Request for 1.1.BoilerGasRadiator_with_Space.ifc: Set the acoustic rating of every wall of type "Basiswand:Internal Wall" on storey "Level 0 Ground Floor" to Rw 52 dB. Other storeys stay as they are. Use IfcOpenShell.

First a look at what the model holds.

```python
import ifcopenshell
import ifcopenshell.util.element

model = ifcopenshell.open("1.1.BoilerGasRadiator_with_Space.ifc")
print(model.schema)
storey = next(s for s in model.by_type("IfcBuildingStorey") if s.Name == "Level 0 Ground Floor")
walls = [e for e in ifcopenshell.util.element.get_decomposition(storey) if e.is_a("IfcWall")]
seen = {}
for e in walls:
    element_type = ifcopenshell.util.element.get_type(e)
    key = (element_type.Name if element_type != e and element_type else None, ifcopenshell.util.element.get_pset(e, "Pset_WallCommon", "AcousticRating"))
    seen[key] = seen.get(key, 0) + 1
for (name, value), count in sorted(seen.items(), key=str):
    print(count, "x", name, "|", value)
```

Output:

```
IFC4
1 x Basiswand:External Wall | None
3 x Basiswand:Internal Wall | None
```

```python
import ifcopenshell
import ifcopenshell.api.pset
import ifcopenshell.util.element

model = ifcopenshell.open("1.1.BoilerGasRadiator_with_Space.ifc")

storey = next(s for s in model.by_type("IfcBuildingStorey") if s.Name == "Level 0 Ground Floor")
walls = [e for e in ifcopenshell.util.element.get_decomposition(storey) if e.is_a("IfcWall")]

count = 0
for e in walls:
    element_type = ifcopenshell.util.element.get_type(e)
    if element_type in (None, e) or element_type.Name != "Basiswand:Internal Wall":
        continue
    # add_pset returns the element's existing set when there is one.
    pset = ifcopenshell.api.pset.add_pset(model, product=e, name="Pset_WallCommon")
    ifcopenshell.api.pset.edit_pset(model, pset=pset, properties={"AcousticRating": "Rw 52 dB"})
    count += 1

print(count, "walls updated")

model.write("1.1.BoilerGasRadiator_with_Space_updated.ifc")
```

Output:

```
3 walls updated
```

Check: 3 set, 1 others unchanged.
